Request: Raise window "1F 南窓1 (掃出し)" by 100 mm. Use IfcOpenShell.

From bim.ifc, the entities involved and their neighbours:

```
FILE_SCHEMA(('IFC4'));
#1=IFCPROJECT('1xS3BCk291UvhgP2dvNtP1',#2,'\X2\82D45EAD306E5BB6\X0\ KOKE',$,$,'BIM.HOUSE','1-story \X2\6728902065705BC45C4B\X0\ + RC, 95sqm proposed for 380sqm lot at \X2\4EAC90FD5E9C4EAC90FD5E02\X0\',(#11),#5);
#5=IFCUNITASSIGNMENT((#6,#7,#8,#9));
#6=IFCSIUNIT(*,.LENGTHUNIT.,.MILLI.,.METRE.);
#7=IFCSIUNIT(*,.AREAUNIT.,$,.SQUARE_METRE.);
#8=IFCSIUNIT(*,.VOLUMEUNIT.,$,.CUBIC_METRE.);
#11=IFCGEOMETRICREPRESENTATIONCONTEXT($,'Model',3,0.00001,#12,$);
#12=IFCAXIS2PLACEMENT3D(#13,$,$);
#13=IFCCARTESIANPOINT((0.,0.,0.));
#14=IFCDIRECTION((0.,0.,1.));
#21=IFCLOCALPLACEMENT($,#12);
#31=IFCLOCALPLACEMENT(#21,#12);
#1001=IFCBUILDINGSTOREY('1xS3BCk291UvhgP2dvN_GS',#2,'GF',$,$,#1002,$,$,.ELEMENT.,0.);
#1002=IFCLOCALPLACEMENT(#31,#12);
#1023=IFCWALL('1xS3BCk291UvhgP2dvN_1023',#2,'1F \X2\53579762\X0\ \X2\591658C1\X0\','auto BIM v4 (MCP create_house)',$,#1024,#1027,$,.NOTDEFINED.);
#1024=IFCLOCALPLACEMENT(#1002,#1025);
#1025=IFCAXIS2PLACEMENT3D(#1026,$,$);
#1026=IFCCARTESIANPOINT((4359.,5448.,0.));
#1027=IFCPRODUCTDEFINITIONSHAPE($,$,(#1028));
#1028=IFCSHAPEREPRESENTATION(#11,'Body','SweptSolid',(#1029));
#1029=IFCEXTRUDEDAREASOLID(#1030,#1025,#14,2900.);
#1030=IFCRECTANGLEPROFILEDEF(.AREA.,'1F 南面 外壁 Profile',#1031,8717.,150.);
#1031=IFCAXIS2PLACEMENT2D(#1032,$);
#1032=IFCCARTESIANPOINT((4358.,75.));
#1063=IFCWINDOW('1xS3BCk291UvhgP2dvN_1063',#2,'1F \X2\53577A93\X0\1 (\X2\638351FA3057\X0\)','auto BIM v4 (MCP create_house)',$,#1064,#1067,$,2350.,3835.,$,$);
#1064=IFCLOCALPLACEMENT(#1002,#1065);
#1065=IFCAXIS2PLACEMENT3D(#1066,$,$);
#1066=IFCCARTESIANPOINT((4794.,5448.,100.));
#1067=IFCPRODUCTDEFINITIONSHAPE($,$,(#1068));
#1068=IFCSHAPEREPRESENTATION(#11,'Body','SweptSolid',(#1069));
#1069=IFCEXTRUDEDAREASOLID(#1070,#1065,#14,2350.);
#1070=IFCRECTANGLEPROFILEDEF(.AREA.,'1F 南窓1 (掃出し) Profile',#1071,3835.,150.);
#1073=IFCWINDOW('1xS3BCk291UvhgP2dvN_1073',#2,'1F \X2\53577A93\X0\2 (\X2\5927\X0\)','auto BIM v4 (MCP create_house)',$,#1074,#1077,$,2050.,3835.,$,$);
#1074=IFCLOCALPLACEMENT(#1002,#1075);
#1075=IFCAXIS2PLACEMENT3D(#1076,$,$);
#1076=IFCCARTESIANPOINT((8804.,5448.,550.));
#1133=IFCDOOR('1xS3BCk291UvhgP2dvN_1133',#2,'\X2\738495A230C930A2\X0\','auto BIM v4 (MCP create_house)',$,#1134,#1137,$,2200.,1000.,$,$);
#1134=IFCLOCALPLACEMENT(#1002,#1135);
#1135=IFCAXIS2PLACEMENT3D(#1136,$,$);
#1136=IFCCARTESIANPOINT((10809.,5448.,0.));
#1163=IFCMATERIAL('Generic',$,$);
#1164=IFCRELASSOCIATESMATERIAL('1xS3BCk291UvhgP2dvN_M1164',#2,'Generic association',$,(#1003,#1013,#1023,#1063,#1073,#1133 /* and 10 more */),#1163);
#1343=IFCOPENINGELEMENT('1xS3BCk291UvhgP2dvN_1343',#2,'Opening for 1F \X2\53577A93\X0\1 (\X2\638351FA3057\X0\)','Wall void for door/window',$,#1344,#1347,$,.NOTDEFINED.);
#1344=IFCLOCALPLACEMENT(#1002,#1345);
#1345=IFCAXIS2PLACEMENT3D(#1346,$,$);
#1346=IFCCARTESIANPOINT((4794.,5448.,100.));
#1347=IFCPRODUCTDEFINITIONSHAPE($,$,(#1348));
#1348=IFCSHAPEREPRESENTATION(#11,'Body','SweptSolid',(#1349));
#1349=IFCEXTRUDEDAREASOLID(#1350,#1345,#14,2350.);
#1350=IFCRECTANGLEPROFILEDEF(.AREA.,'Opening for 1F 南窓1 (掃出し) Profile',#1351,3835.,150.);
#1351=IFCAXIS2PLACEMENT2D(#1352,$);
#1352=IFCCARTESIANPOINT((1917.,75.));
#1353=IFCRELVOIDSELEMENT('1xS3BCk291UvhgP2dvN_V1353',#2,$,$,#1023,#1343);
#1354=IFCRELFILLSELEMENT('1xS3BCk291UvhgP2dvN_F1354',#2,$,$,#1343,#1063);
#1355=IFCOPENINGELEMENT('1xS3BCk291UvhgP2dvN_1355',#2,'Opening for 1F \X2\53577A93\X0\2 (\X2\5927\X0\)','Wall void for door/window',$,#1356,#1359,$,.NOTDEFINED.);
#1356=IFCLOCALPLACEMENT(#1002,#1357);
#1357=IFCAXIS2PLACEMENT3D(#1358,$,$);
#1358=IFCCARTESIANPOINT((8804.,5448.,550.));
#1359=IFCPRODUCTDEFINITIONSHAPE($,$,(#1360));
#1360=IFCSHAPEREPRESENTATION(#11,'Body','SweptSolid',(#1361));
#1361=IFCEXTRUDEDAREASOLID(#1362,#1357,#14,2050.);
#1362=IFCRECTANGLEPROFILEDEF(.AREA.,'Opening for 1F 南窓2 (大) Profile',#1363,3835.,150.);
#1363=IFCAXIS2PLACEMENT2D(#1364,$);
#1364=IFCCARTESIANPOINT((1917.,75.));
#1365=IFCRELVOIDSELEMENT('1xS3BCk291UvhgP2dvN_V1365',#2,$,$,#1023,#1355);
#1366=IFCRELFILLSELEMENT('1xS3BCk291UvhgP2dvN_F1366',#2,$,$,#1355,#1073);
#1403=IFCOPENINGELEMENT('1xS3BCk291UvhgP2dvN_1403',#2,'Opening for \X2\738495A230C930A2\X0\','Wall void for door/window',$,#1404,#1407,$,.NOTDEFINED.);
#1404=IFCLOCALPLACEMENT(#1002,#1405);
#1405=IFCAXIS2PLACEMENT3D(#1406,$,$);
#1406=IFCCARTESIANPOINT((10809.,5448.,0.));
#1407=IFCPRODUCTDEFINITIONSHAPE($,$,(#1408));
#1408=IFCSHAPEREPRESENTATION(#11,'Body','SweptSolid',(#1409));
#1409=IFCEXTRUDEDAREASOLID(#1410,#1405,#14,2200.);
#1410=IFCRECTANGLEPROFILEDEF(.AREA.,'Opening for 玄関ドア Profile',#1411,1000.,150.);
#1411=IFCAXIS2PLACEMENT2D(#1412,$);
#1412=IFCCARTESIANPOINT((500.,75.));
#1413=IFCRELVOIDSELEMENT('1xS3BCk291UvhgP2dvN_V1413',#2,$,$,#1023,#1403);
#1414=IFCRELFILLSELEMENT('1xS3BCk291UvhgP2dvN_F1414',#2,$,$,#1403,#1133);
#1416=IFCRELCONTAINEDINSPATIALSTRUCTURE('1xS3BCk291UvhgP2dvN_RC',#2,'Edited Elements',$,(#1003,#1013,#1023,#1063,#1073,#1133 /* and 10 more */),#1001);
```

```python
import numpy as np
import ifcopenshell
import ifcopenshell.api.geometry
import ifcopenshell.util.placement
import ifcopenshell.util.unit

model = ifcopenshell.open("bim.ifc")
unit_scale = ifcopenshell.util.unit.calculate_unit_scale(model)

window = model.by_guid("1xS3BCk291UvhgP2dvN_1063")
opening = window.FillsVoids[0].RelatingOpeningElement
dz = 0.1 / unit_scale

shift = np.array([0.0, 0.0, dz])
# The window is not placed relative to its opening, so move both.
for product in (opening, window):
    matrix = ifcopenshell.util.placement.get_local_placement(product.ObjectPlacement)
    matrix[:3, 3] += shift
    ifcopenshell.api.geometry.edit_object_placement(model, product=product, matrix=matrix, is_si=False)

print(f"moved by {dz * unit_scale:+.3f} m")

model.write("bim_updated.ifc")
```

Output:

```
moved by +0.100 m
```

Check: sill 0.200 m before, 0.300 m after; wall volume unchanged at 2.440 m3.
